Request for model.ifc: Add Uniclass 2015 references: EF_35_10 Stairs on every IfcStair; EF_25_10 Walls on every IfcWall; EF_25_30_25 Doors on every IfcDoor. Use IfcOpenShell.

First a look at what the model holds.

```python
import ifcopenshell

model = ifcopenshell.open("model.ifc")
print(model.schema)
print("classifications:", [c.Name for c in model.by_type("IfcClassification")])
for ifc_class in ("IfcDoor", "IfcRoof", "IfcStair", "IfcWall", "IfcWindow"):
    print(ifc_class, len(model.by_type(ifc_class)))
```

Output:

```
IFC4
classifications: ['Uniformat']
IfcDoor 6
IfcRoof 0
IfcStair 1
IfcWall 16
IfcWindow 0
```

```python
import ifcopenshell
import ifcopenshell.api.classification

model = ifcopenshell.open("model.ifc")

system = ifcopenshell.api.classification.add_classification(model, classification="Uniclass 2015")

codes = {
    "IfcStair": ("EF_35_10", "Stairs"),
    "IfcWall": ("EF_25_10", "Walls"),
    "IfcDoor": ("EF_25_30_25", "Doors"),
}
for ifc_class, (code, name) in codes.items():
    products = model.by_type(ifc_class)
    ifcopenshell.api.classification.add_reference(
        model, products=products, classification=system, identification=code, name=name
    )
    print(code, len(products))

model.write("model_updated.ifc")
```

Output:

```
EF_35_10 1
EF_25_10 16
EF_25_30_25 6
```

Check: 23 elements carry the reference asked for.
